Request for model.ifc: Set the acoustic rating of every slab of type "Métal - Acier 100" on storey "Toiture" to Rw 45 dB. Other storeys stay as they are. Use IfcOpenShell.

First a look at what the model holds.

```python
import ifcopenshell
import ifcopenshell.util.element

model = ifcopenshell.open("model.ifc")
print(model.schema)
storey = next(s for s in model.by_type("IfcBuildingStorey") if s.Name == "Toiture")
slabs = [e for e in ifcopenshell.util.element.get_decomposition(storey) if e.is_a("IfcSlab")]
seen = {}
for e in slabs:
    element_type = ifcopenshell.util.element.get_type(e)
    key = (element_type.Name if element_type != e and element_type else None, ifcopenshell.util.element.get_pset(e, "Pset_SlabCommon", "AcousticRating"))
    seen[key] = seen.get(key, 0) + 1
for (name, value), count in sorted(seen.items(), key=str):
    print(count, "x", name, "|", value)
```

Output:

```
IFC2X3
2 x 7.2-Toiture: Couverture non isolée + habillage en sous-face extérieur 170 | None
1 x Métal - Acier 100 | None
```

```python
import ifcopenshell
import ifcopenshell.api.pset
import ifcopenshell.util.element

model = ifcopenshell.open("model.ifc")

storey = next(s for s in model.by_type("IfcBuildingStorey") if s.Name == "Toiture")
slabs = [e for e in ifcopenshell.util.element.get_decomposition(storey) if e.is_a("IfcSlab")]

count = 0
for e in slabs:
    element_type = ifcopenshell.util.element.get_type(e)
    if element_type in (None, e) or element_type.Name != "Métal - Acier 100":
        continue
    # add_pset returns the element's existing set when there is one.
    pset = ifcopenshell.api.pset.add_pset(model, product=e, name="Pset_SlabCommon")
    ifcopenshell.api.pset.edit_pset(model, pset=pset, properties={"AcousticRating": "Rw 45 dB"})
    count += 1

print(count, "slabs updated")

model.write("model_edited.ifc")
```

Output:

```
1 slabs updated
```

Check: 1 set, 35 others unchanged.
